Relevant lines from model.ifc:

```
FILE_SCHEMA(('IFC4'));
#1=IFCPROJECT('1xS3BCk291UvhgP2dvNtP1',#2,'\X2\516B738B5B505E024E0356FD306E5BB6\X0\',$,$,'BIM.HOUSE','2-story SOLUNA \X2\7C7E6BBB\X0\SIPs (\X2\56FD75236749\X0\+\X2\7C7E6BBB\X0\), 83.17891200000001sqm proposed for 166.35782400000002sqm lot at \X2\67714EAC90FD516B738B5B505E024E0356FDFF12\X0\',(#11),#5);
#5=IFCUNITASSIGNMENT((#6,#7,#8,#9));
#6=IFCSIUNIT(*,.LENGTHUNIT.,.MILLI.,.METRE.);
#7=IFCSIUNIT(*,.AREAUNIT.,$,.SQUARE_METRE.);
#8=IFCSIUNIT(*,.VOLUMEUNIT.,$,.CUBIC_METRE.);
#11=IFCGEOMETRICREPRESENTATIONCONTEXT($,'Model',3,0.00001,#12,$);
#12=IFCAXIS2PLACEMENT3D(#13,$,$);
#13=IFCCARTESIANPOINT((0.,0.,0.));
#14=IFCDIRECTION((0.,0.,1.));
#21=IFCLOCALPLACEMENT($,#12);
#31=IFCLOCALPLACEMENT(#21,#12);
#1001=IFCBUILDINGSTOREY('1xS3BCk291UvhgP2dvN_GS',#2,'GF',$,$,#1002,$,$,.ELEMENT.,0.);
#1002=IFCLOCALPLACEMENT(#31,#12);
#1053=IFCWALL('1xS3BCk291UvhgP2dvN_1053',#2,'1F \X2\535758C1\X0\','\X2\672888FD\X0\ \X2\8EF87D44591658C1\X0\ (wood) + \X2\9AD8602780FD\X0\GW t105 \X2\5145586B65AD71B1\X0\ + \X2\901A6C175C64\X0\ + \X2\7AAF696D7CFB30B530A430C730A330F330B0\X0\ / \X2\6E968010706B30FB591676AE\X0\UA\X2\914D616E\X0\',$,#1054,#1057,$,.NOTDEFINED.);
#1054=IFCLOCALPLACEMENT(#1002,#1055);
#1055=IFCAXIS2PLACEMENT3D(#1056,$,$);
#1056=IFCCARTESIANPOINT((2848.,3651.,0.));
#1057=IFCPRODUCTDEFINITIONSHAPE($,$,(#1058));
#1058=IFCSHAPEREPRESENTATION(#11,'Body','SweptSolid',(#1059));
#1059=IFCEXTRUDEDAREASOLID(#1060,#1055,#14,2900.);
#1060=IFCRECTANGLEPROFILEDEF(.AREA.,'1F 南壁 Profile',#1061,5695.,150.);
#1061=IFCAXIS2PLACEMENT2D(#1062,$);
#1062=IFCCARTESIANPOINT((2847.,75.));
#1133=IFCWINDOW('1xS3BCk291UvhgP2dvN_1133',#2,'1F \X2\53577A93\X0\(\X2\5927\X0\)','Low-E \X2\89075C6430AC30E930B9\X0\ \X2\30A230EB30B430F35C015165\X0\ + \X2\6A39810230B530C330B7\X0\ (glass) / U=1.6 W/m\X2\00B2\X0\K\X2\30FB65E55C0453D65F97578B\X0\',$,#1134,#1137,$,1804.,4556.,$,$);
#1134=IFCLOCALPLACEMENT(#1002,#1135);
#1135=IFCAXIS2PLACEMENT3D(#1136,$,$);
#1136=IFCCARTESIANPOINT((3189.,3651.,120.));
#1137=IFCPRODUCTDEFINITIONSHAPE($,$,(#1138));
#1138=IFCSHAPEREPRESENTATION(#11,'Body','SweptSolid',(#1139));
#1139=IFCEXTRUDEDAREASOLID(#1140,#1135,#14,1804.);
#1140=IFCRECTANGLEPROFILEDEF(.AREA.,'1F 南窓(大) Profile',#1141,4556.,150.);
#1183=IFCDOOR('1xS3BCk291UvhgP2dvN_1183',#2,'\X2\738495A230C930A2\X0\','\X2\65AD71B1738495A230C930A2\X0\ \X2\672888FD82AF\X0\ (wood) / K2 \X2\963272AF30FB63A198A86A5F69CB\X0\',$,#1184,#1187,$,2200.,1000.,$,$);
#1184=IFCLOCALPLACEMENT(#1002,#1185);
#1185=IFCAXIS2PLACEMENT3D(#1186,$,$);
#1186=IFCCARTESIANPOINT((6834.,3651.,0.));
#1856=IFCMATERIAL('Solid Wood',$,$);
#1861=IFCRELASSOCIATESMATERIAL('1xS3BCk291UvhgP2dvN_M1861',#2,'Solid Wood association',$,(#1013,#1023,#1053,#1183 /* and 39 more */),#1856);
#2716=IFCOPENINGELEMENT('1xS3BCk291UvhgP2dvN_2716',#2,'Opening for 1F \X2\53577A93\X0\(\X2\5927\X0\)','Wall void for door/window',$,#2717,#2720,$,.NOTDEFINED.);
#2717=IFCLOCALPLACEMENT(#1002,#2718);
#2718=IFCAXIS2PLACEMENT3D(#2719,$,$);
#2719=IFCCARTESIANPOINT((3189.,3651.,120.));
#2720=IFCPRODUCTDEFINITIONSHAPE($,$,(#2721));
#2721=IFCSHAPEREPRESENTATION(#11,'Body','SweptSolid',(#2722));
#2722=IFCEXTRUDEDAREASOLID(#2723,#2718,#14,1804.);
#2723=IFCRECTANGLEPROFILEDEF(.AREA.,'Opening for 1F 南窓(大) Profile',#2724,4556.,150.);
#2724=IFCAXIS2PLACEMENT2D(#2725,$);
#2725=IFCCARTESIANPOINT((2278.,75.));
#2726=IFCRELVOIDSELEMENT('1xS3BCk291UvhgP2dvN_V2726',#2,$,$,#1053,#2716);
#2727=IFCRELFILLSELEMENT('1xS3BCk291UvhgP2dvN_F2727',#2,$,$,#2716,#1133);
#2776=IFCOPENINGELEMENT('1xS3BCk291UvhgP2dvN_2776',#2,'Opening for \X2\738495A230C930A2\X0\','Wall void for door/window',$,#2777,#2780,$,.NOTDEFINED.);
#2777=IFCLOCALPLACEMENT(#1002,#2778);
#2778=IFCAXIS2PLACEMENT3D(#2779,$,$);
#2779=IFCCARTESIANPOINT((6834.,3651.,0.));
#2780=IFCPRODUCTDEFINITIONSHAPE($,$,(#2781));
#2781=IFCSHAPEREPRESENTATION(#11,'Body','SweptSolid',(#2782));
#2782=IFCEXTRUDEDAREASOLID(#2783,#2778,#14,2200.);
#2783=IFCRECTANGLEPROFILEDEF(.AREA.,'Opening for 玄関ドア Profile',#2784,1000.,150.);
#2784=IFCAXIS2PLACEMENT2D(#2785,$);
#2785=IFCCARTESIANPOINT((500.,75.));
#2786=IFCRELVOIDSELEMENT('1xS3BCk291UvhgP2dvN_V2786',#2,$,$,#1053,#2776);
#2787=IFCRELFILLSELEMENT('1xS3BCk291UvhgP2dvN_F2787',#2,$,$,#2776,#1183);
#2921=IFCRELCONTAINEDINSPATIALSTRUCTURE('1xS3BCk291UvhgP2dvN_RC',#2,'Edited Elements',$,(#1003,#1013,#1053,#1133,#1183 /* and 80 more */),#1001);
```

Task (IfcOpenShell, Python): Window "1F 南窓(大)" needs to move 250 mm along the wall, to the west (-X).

```python
import ifcopenshell
import ifcopenshell.api.geometry
import ifcopenshell.util.placement
import ifcopenshell.util.unit

model = ifcopenshell.open("model.ifc")
unit_scale = ifcopenshell.util.unit.calculate_unit_scale(model)

window = model.by_guid("1xS3BCk291UvhgP2dvN_1133")
opening = window.FillsVoids[0].RelatingOpeningElement
wall = opening.VoidsElements[0].RelatingBuildingElement

wall_matrix = ifcopenshell.util.placement.get_local_placement(wall.ObjectPlacement)
shift = wall_matrix[:3, 0] * -0.25 / unit_scale
before = ifcopenshell.util.placement.get_local_placement(window.ObjectPlacement)[:3, 3].copy()

# The window is not placed relative to its opening, so move both.
for product in (opening, window):
    matrix = ifcopenshell.util.placement.get_local_placement(product.ObjectPlacement)
    matrix[:3, 3] += shift
    ifcopenshell.api.geometry.edit_object_placement(model, product=product, matrix=matrix, is_si=False)

after = ifcopenshell.util.placement.get_local_placement(window.ObjectPlacement)[:3, 3]
print("window moved by", (after - before).round(3) + 0.0)

model.write("model_v2.ifc")
```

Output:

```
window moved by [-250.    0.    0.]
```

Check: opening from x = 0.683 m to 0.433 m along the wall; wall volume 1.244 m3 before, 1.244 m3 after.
